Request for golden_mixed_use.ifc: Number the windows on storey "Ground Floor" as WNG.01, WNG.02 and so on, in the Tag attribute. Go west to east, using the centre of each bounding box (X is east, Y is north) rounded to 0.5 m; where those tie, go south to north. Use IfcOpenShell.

First a look at what the model holds.

```python
import ifcopenshell
import ifcopenshell.util.element
import ifcopenshell.util.placement

model = ifcopenshell.open("golden_mixed_use.ifc")
print(model.schema)
storey = next(s for s in model.by_type("IfcBuildingStorey") if s.Name == "Ground Floor")
windows = [e for e in ifcopenshell.util.element.get_decomposition(storey) if e.is_a("IfcWindow")]
for e in sorted(windows, key=lambda e: e.id()):
    origin = ifcopenshell.util.placement.get_local_placement(e.ObjectPlacement)[:3, 3]
    print(e.id(), e.Tag, e.Name, origin.round(2) + 0.0, sep=" | ")
```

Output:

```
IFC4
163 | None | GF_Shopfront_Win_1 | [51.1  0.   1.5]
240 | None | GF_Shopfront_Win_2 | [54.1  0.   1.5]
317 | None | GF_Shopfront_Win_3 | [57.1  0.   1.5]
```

```python
import ifcopenshell
import ifcopenshell.geom
import ifcopenshell.util.element
import ifcopenshell.util.shape

model = ifcopenshell.open("golden_mixed_use.ifc")
settings = ifcopenshell.geom.settings()
settings.set("use-world-coords", True)


def centre(element):
    shape = ifcopenshell.geom.create_shape(settings, element)
    return ifcopenshell.util.shape.get_bbox_centroid(shape.geometry)


storey = next(s for s in model.by_type("IfcBuildingStorey") if s.Name == "Ground Floor")
windows = [e for e in ifcopenshell.util.element.get_decomposition(storey) if e.is_a("IfcWindow")]

# Insertion points can sit at a corner or the storey origin, so sort by the geometry (in metres).
centres = {e: centre(e) for e in windows}
windows.sort(key=lambda e: (round(centres[e][0] / 0.5), centres[e][1]))

for i, e in enumerate(windows, start=1):
    number = f"WNG.{i:02d}"
    e.Tag = number
    print(e.id(), number)

model.write("golden_mixed_use_updated.ifc")
```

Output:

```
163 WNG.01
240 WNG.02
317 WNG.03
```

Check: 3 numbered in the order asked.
